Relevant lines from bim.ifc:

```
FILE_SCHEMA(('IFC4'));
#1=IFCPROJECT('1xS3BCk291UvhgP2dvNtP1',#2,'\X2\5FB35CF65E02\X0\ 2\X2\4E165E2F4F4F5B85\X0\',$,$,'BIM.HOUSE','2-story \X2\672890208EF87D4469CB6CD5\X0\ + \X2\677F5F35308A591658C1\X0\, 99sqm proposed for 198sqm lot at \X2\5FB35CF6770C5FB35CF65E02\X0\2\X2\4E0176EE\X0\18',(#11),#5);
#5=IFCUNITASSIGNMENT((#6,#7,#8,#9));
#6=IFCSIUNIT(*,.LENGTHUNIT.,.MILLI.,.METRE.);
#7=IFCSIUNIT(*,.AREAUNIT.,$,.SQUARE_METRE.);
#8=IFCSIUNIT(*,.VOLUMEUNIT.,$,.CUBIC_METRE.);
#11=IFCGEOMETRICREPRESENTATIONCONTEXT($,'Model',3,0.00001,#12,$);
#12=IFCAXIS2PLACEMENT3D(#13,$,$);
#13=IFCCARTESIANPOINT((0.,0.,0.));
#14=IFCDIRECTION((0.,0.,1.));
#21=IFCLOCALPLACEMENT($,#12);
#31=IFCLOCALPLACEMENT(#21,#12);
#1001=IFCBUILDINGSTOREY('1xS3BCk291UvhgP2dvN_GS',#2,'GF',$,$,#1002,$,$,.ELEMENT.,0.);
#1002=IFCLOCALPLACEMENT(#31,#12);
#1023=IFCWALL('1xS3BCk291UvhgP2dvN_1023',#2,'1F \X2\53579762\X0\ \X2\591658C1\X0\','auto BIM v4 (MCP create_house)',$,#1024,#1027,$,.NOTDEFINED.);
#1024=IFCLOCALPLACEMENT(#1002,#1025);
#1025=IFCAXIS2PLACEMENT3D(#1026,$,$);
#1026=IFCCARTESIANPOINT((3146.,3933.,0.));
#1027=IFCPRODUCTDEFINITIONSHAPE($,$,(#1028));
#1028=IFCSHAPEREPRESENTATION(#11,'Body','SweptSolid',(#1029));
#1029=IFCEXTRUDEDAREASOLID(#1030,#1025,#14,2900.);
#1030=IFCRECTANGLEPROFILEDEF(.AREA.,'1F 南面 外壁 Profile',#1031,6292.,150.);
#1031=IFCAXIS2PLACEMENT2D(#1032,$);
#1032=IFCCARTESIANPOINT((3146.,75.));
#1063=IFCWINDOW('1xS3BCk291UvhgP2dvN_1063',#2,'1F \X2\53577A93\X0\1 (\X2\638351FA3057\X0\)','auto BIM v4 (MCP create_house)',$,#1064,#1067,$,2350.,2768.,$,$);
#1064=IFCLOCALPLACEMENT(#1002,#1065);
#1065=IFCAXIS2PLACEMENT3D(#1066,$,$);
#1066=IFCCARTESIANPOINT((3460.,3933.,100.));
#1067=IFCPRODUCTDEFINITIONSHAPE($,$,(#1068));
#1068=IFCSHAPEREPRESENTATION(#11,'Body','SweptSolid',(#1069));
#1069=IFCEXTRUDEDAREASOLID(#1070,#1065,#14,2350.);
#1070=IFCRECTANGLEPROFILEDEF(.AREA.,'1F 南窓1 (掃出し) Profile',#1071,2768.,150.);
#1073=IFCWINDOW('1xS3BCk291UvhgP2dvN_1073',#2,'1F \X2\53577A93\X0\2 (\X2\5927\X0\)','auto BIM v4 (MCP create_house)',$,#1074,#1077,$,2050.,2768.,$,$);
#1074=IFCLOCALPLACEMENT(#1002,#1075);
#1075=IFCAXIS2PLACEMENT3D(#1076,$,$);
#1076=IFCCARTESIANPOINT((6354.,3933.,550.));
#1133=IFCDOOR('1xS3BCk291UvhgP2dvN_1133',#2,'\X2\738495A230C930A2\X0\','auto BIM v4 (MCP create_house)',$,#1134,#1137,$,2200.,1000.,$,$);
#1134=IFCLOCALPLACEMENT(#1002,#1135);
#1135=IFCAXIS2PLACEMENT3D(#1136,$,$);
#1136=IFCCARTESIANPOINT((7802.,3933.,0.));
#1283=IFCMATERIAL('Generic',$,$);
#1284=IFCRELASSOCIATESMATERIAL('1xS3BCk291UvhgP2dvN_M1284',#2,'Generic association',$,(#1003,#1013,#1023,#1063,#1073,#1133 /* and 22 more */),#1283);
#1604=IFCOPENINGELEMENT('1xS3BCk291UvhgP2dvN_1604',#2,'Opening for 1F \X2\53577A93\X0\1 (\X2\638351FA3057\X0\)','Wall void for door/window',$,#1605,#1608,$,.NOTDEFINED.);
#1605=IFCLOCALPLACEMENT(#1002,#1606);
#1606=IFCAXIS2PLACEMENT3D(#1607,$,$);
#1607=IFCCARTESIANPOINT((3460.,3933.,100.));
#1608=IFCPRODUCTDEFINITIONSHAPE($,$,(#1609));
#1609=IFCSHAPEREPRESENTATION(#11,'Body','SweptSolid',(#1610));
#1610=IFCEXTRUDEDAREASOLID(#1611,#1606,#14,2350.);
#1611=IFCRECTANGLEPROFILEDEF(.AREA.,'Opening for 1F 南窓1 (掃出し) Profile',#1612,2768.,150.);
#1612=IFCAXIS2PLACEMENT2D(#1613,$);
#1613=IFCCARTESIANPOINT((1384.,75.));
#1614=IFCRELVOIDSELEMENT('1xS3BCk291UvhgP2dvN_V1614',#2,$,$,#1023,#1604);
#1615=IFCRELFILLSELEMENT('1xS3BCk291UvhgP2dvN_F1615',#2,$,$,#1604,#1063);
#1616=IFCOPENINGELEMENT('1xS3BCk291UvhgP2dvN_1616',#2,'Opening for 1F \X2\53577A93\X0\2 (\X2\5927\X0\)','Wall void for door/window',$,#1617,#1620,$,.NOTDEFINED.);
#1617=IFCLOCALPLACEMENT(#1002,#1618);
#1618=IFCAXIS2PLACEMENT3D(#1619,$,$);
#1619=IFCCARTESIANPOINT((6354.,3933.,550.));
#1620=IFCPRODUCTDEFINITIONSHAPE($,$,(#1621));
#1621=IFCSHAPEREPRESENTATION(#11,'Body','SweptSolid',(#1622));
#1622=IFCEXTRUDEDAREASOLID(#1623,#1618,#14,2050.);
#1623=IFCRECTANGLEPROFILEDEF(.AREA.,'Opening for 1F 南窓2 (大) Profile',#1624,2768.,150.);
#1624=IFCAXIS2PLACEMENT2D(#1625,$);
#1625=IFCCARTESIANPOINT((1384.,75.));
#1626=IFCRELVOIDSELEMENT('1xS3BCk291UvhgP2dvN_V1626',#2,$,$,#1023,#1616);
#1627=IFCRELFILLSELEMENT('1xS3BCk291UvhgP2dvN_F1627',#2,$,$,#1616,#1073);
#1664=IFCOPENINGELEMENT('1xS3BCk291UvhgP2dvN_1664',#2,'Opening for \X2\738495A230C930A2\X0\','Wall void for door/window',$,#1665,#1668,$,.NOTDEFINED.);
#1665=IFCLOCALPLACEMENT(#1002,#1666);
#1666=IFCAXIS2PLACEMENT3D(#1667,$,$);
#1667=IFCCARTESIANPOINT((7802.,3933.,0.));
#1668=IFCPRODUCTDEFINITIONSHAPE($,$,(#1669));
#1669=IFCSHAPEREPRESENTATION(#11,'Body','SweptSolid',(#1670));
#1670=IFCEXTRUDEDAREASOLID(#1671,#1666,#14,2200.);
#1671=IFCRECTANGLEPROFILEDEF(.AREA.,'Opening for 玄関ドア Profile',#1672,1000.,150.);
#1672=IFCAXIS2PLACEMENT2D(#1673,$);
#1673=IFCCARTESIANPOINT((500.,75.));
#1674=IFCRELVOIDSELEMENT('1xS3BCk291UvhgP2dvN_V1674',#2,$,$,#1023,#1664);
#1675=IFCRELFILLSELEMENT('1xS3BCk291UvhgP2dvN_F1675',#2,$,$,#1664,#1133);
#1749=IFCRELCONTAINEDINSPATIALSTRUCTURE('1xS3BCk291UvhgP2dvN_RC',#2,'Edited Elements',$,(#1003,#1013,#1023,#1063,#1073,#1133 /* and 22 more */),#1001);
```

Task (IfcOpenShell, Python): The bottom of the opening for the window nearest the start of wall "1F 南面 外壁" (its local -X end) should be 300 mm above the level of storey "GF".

```python
import numpy as np
import ifcopenshell
import ifcopenshell.api.geometry
import ifcopenshell.geom
import ifcopenshell.util.element
import ifcopenshell.util.placement
import ifcopenshell.util.shape
import ifcopenshell.util.unit

model = ifcopenshell.open("bim.ifc")
unit_scale = ifcopenshell.util.unit.calculate_unit_scale(model)

window = model.by_id(1063)
opening = window.FillsVoids[0].RelatingOpeningElement
storey = ifcopenshell.util.element.get_container(window, ifc_class="IfcBuildingStorey")
level = ifcopenshell.util.placement.get_local_placement(storey.ObjectPlacement)[2, 3]

# The opening's origin need not be at the sill, so measure its lowest point.
shape = ifcopenshell.geom.create_shape(ifcopenshell.geom.settings(), opening)
bottom = ifcopenshell.util.shape.get_shape_bottom_elevation(shape, shape.geometry) / unit_scale
dz = level + 0.3 / unit_scale - bottom

shift = np.array([0.0, 0.0, dz])
# The window is not placed relative to its opening, so move both.
for product in (opening, window):
    matrix = ifcopenshell.util.placement.get_local_placement(product.ObjectPlacement)
    matrix[:3, 3] += shift
    ifcopenshell.api.geometry.edit_object_placement(model, product=product, matrix=matrix, is_si=False)

print(f"moved by {dz * unit_scale:+.3f} m")

model.write("bim_edited.ifc")
```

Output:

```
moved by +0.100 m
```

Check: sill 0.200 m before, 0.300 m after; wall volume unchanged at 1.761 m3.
